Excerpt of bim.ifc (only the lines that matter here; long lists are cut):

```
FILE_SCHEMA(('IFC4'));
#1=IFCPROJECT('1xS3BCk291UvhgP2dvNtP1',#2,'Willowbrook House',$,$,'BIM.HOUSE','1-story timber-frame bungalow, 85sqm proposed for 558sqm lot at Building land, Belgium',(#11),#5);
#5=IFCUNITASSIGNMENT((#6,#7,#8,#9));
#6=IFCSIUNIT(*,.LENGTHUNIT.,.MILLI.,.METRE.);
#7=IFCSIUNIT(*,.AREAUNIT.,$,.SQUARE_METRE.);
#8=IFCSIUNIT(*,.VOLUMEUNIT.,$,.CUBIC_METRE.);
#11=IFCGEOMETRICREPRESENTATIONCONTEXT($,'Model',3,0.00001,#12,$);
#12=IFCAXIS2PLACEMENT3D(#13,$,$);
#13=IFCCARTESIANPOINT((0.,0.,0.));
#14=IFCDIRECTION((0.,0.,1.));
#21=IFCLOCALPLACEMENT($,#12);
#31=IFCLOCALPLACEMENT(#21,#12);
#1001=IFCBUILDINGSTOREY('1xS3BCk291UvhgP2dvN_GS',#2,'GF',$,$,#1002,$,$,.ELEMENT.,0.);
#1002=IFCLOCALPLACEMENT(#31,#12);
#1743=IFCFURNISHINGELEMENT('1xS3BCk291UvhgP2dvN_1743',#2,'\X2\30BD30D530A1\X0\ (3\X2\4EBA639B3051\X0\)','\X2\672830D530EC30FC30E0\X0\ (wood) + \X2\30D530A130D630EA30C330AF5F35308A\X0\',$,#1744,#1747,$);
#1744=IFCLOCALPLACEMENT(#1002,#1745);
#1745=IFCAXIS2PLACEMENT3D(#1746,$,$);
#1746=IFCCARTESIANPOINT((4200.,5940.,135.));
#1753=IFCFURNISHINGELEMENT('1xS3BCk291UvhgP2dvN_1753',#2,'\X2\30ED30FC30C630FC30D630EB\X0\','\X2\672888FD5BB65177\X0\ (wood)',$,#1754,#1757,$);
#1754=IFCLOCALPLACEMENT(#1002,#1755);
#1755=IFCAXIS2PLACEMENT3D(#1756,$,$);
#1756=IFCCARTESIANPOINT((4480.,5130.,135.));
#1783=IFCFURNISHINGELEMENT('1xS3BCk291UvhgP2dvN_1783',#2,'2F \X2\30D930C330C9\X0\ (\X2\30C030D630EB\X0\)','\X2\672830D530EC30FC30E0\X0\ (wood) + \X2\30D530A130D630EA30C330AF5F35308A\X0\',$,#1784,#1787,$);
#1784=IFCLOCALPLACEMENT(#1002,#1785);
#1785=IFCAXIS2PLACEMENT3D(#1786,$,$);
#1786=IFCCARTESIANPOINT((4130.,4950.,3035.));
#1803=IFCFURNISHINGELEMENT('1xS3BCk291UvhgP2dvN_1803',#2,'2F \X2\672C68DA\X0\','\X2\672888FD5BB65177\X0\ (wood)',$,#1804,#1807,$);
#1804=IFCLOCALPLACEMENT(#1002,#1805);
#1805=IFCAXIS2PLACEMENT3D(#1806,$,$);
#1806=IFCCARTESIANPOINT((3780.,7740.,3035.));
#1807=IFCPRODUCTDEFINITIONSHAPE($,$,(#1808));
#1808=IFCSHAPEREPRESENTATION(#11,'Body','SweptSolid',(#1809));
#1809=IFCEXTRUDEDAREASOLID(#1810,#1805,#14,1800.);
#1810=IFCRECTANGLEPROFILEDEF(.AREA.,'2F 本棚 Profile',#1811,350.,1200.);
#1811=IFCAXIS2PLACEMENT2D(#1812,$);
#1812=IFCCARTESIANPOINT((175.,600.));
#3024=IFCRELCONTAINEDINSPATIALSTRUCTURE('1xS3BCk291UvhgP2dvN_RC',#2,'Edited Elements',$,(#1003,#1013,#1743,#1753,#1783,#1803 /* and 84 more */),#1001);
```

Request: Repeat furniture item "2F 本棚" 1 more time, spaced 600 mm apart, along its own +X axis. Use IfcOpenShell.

```python
import ifcopenshell
import ifcopenshell.api.geometry
import ifcopenshell.api.root
import ifcopenshell.util.element
import ifcopenshell.util.placement

model = ifcopenshell.open("bim.ifc")


def reuse_history(source, copy):
    """copy_class also copies each property set's owner history, people and application; keep the originals."""
    for rel in copy.IsDefinedBy:
        if rel.is_a("IfcRelDefinesByProperties") and (history := rel.RelatingPropertyDefinition.OwnerHistory):
            rel.RelatingPropertyDefinition.OwnerHistory = source.OwnerHistory
            ifcopenshell.util.element.remove_deep2(model, history)


source = model.by_guid("1xS3BCk291UvhgP2dvN_1803")
base = ifcopenshell.util.placement.get_local_placement(source.ObjectPlacement)
step = base[:3, 0] * 600.0

for i in range(1, 2):
    copy = ifcopenshell.api.root.copy_class(model, product=source)
    copy.Representation = ifcopenshell.util.element.copy_deep(
        model, source.Representation, exclude=["IfcGeometricRepresentationContext", "IfcRepresentationMap"]
    )
    reuse_history(source, copy)
    matrix = base.copy()
    matrix[:3, 3] += i * step
    print("added at", matrix[:3, 3].round(3) + 0.0)
    ifcopenshell.api.geometry.edit_object_placement(model, product=copy, matrix=matrix, is_si=False)

model.write("bim_v2.ifc")
```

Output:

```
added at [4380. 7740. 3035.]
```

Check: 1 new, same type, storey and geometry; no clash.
